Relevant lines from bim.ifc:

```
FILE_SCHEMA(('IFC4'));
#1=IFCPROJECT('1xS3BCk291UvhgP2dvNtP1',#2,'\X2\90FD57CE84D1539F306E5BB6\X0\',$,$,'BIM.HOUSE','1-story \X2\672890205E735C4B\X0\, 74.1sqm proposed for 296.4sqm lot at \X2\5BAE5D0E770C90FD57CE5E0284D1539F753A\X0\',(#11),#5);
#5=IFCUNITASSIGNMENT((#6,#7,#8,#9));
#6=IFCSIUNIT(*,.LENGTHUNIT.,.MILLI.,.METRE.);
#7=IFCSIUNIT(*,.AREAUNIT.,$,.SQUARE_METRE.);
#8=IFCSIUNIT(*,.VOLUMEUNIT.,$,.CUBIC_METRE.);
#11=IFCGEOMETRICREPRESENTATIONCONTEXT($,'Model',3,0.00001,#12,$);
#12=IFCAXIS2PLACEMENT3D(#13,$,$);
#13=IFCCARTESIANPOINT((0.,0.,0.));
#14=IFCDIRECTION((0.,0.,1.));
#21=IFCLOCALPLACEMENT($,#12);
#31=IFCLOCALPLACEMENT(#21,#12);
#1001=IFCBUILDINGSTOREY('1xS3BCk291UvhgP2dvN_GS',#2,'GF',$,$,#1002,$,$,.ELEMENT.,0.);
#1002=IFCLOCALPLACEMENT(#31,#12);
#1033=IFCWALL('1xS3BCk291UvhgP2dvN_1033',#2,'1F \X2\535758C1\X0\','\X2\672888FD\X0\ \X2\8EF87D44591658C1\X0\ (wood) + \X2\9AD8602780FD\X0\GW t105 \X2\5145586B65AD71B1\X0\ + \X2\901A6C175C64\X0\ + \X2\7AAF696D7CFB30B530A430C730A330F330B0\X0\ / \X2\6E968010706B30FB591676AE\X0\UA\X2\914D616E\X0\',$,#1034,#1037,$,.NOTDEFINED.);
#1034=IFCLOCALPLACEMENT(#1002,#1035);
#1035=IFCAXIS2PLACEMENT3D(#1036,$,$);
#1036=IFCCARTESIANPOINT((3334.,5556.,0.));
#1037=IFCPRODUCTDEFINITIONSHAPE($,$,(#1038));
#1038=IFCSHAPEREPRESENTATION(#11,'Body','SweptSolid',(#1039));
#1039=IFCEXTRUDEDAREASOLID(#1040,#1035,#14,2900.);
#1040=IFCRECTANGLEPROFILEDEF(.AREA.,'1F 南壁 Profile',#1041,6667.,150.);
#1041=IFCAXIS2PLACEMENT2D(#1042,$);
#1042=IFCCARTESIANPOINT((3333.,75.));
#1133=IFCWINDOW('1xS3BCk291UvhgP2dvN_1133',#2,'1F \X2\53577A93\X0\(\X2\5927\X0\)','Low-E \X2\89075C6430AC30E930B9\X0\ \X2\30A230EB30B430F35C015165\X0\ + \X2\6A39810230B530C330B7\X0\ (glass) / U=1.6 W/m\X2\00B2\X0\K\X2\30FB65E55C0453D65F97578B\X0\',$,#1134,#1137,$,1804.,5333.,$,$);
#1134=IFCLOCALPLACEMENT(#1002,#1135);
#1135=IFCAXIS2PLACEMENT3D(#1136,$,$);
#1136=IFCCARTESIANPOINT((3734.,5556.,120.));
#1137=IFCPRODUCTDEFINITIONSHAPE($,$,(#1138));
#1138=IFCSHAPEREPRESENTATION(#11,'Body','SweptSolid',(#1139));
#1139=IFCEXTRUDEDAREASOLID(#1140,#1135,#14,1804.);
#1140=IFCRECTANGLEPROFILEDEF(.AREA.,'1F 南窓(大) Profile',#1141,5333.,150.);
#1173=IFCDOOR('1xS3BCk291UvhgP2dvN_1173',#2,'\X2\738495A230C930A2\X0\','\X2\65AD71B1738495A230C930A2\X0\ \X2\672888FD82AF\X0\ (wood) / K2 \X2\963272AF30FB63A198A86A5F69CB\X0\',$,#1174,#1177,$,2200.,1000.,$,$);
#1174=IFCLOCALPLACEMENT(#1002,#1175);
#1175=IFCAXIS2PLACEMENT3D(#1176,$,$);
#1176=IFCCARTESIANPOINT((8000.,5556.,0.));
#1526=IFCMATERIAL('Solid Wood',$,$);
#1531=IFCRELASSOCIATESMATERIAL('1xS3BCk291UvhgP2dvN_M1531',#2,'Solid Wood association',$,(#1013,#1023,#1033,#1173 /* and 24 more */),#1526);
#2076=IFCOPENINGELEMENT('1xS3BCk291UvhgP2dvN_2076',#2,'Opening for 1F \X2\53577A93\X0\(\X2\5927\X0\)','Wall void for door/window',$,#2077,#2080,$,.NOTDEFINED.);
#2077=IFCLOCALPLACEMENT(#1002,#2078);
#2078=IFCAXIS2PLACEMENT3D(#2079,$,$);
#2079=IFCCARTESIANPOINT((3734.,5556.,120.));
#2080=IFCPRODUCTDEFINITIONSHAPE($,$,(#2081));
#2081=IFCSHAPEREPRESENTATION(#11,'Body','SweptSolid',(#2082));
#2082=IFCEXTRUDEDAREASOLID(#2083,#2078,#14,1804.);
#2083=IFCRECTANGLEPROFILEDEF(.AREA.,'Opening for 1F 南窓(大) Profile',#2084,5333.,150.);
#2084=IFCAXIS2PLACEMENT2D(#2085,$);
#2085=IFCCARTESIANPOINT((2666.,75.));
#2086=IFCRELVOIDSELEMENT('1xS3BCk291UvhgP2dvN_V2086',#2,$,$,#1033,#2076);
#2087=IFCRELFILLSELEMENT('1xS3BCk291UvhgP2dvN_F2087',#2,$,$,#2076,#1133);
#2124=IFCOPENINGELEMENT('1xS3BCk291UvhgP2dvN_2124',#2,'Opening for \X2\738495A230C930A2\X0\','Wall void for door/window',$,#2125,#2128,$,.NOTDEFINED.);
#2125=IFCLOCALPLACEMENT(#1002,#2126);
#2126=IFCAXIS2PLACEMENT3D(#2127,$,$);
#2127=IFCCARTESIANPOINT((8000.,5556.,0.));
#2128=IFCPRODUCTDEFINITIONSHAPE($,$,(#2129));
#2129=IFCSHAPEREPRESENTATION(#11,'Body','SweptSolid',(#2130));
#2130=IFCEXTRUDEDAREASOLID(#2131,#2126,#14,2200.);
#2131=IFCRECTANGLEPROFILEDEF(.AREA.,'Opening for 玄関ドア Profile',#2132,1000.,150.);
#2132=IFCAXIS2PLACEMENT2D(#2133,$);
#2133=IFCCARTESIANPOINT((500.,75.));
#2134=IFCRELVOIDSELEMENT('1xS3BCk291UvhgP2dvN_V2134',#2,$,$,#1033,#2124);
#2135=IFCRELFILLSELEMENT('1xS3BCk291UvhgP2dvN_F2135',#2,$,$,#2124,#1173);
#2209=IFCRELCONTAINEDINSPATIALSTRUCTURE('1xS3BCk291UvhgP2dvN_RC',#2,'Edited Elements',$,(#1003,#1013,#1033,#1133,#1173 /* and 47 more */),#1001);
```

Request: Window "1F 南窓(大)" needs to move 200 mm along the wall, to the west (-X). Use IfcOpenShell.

```python
import ifcopenshell
import ifcopenshell.api.geometry
import ifcopenshell.util.placement

model = ifcopenshell.open("bim.ifc")

window = model.by_guid("1xS3BCk291UvhgP2dvN_1133")
opening = window.FillsVoids[0].RelatingOpeningElement
wall = opening.VoidsElements[0].RelatingBuildingElement

wall_matrix = ifcopenshell.util.placement.get_local_placement(wall.ObjectPlacement)
shift = wall_matrix[:3, 0] * -200.0
before = ifcopenshell.util.placement.get_local_placement(window.ObjectPlacement)[:3, 3].copy()

# The window is not placed relative to its opening, so move both.
for product in (opening, window):
    matrix = ifcopenshell.util.placement.get_local_placement(product.ObjectPlacement)
    matrix[:3, 3] += shift
    ifcopenshell.api.geometry.edit_object_placement(model, product=product, matrix=matrix, is_si=False)

after = ifcopenshell.util.placement.get_local_placement(window.ObjectPlacement)[:3, 3]
print("window moved by", (after - before).round(3) + 0.0)

model.write("bim_updated.ifc")
```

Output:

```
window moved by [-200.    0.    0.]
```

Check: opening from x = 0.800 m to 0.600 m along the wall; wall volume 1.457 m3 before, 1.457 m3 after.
